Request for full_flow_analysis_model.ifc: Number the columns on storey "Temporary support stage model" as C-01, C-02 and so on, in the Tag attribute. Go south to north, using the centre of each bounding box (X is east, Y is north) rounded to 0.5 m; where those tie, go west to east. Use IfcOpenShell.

First a look at what the model holds.

```python
import ifcopenshell
import ifcopenshell.util.element
import ifcopenshell.util.placement

model = ifcopenshell.open("full_flow_analysis_model.ifc")
print(model.schema)
storey = next(s for s in model.by_type("IfcBuildingStorey") if s.Name == "Temporary support stage model")
columns = [e for e in ifcopenshell.util.element.get_decomposition(storey) if e.is_a("IfcColumn")]
for e in sorted(columns, key=lambda e: e.id()):
    origin = ifcopenshell.util.placement.get_local_placement(e.ObjectPlacement)[:3, 3]
    print(e.id(), e.Tag, e.Name, origin.round(2) + 0.0, sep=" | ")
```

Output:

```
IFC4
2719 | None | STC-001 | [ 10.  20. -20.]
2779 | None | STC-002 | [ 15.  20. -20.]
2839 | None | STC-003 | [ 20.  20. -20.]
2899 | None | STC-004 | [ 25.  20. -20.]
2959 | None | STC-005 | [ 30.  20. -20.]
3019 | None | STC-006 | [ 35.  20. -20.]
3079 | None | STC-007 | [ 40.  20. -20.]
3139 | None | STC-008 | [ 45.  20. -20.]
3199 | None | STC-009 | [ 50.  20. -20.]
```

```python
import ifcopenshell
import ifcopenshell.geom
import ifcopenshell.util.element
import ifcopenshell.util.shape

model = ifcopenshell.open("full_flow_analysis_model.ifc")
settings = ifcopenshell.geom.settings()
settings.set("use-world-coords", True)


def centre(element):
    shape = ifcopenshell.geom.create_shape(settings, element)
    return ifcopenshell.util.shape.get_bbox_centroid(shape.geometry)


storey = next(s for s in model.by_type("IfcBuildingStorey") if s.Name == "Temporary support stage model")
columns = [e for e in ifcopenshell.util.element.get_decomposition(storey) if e.is_a("IfcColumn")]

# Insertion points can sit at a corner or the storey origin, so sort by the geometry (in metres).
centres = {e: centre(e) for e in columns}
columns.sort(key=lambda e: (round(centres[e][1] / 0.5), centres[e][0]))

for i, e in enumerate(columns, start=1):
    number = f"C-{i:02d}"
    e.Tag = number
    print(e.id(), number)

model.write("full_flow_analysis_model_edited.ifc")
```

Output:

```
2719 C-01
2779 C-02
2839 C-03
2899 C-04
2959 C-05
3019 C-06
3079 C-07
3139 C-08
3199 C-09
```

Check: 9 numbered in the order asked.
